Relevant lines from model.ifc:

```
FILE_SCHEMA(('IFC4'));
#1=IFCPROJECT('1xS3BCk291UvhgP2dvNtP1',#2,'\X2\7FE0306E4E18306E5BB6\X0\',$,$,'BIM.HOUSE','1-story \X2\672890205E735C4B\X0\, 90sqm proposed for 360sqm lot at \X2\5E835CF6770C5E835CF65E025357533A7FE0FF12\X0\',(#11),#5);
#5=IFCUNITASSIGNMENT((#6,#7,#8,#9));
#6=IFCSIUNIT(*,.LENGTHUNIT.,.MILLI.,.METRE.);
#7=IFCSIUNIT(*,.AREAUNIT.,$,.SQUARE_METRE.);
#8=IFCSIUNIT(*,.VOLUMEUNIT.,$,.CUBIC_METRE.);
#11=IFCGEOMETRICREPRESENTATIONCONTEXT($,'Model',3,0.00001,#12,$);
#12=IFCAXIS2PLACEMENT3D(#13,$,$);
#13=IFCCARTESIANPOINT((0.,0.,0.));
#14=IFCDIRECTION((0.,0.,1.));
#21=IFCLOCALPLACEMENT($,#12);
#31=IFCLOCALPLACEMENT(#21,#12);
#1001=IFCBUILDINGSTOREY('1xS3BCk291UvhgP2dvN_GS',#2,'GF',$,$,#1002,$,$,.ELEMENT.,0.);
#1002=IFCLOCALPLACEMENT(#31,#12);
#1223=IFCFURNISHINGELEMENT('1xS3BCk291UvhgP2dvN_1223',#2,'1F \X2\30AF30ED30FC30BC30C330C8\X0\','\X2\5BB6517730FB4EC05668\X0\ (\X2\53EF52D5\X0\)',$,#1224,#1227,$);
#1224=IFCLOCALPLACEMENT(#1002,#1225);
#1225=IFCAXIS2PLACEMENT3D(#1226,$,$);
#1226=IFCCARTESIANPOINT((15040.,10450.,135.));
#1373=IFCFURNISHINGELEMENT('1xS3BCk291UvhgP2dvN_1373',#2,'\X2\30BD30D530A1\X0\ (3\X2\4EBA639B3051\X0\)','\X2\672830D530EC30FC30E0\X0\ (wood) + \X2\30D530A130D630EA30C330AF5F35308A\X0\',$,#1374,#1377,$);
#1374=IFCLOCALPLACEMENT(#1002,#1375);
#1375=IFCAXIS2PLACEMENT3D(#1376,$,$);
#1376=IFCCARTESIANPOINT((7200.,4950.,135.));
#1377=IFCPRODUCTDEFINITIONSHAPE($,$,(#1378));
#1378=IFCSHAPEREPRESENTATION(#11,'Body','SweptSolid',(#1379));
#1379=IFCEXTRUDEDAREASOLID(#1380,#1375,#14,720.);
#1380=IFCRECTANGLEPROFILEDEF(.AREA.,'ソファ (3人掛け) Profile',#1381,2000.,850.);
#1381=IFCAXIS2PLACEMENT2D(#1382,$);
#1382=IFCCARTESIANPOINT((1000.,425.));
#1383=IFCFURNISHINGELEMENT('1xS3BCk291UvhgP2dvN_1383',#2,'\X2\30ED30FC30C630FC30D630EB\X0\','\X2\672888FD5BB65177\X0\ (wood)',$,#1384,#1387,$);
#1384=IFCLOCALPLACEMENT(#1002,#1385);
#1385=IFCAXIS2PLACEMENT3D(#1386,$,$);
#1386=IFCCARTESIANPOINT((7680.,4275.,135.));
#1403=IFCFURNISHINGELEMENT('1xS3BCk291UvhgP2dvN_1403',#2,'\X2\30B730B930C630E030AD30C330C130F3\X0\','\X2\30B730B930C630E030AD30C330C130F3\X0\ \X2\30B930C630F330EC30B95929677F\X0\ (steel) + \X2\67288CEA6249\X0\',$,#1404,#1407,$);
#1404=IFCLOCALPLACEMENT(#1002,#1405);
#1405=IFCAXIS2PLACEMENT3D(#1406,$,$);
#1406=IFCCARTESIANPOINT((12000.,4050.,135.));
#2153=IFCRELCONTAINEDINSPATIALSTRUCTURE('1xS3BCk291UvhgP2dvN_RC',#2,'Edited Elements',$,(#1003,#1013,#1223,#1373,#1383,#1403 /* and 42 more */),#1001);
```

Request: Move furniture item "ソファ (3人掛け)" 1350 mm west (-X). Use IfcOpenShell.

```python
import ifcopenshell
import ifcopenshell.api.geometry
import ifcopenshell.util.placement
import ifcopenshell.util.unit

model = ifcopenshell.open("model.ifc")
unit_scale = ifcopenshell.util.unit.calculate_unit_scale(model)

item = model.by_guid("1xS3BCk291UvhgP2dvN_1373")
matrix = ifcopenshell.util.placement.get_local_placement(item.ObjectPlacement)
matrix[0, 3] -= 1.35 / unit_scale
ifcopenshell.api.geometry.edit_object_placement(model, product=item, matrix=matrix, is_si=False)

print(ifcopenshell.util.placement.get_local_placement(item.ObjectPlacement).round(3) + 0.0)

model.write("model_edited.ifc")
```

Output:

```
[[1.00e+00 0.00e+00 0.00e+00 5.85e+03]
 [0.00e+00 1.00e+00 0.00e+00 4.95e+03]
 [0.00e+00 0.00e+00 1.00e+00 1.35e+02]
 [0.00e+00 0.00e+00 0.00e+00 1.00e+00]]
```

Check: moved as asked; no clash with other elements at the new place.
